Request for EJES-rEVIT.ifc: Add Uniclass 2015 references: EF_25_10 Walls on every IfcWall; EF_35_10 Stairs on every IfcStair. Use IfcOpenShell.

First a look at what the model holds.

```python
import ifcopenshell

model = ifcopenshell.open("EJES-rEVIT.ifc")
print(model.schema)
print("classifications:", [c.Name for c in model.by_type("IfcClassification")])
for ifc_class in ("IfcDoor", "IfcRoof", "IfcStair", "IfcWall", "IfcWindow"):
    print(ifc_class, len(model.by_type(ifc_class)))
```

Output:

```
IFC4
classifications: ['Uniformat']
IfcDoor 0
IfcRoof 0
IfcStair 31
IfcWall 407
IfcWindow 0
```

```python
import ifcopenshell
import ifcopenshell.api.classification

model = ifcopenshell.open("EJES-rEVIT.ifc")

system = ifcopenshell.api.classification.add_classification(model, classification="Uniclass 2015")

codes = {
    "IfcWall": ("EF_25_10", "Walls"),
    "IfcStair": ("EF_35_10", "Stairs"),
}
for ifc_class, (code, name) in codes.items():
    products = model.by_type(ifc_class)
    ifcopenshell.api.classification.add_reference(
        model, products=products, classification=system, identification=code, name=name
    )
    print(code, len(products))

model.write("EJES-rEVIT_updated.ifc")
```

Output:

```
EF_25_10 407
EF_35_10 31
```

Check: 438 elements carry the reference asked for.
